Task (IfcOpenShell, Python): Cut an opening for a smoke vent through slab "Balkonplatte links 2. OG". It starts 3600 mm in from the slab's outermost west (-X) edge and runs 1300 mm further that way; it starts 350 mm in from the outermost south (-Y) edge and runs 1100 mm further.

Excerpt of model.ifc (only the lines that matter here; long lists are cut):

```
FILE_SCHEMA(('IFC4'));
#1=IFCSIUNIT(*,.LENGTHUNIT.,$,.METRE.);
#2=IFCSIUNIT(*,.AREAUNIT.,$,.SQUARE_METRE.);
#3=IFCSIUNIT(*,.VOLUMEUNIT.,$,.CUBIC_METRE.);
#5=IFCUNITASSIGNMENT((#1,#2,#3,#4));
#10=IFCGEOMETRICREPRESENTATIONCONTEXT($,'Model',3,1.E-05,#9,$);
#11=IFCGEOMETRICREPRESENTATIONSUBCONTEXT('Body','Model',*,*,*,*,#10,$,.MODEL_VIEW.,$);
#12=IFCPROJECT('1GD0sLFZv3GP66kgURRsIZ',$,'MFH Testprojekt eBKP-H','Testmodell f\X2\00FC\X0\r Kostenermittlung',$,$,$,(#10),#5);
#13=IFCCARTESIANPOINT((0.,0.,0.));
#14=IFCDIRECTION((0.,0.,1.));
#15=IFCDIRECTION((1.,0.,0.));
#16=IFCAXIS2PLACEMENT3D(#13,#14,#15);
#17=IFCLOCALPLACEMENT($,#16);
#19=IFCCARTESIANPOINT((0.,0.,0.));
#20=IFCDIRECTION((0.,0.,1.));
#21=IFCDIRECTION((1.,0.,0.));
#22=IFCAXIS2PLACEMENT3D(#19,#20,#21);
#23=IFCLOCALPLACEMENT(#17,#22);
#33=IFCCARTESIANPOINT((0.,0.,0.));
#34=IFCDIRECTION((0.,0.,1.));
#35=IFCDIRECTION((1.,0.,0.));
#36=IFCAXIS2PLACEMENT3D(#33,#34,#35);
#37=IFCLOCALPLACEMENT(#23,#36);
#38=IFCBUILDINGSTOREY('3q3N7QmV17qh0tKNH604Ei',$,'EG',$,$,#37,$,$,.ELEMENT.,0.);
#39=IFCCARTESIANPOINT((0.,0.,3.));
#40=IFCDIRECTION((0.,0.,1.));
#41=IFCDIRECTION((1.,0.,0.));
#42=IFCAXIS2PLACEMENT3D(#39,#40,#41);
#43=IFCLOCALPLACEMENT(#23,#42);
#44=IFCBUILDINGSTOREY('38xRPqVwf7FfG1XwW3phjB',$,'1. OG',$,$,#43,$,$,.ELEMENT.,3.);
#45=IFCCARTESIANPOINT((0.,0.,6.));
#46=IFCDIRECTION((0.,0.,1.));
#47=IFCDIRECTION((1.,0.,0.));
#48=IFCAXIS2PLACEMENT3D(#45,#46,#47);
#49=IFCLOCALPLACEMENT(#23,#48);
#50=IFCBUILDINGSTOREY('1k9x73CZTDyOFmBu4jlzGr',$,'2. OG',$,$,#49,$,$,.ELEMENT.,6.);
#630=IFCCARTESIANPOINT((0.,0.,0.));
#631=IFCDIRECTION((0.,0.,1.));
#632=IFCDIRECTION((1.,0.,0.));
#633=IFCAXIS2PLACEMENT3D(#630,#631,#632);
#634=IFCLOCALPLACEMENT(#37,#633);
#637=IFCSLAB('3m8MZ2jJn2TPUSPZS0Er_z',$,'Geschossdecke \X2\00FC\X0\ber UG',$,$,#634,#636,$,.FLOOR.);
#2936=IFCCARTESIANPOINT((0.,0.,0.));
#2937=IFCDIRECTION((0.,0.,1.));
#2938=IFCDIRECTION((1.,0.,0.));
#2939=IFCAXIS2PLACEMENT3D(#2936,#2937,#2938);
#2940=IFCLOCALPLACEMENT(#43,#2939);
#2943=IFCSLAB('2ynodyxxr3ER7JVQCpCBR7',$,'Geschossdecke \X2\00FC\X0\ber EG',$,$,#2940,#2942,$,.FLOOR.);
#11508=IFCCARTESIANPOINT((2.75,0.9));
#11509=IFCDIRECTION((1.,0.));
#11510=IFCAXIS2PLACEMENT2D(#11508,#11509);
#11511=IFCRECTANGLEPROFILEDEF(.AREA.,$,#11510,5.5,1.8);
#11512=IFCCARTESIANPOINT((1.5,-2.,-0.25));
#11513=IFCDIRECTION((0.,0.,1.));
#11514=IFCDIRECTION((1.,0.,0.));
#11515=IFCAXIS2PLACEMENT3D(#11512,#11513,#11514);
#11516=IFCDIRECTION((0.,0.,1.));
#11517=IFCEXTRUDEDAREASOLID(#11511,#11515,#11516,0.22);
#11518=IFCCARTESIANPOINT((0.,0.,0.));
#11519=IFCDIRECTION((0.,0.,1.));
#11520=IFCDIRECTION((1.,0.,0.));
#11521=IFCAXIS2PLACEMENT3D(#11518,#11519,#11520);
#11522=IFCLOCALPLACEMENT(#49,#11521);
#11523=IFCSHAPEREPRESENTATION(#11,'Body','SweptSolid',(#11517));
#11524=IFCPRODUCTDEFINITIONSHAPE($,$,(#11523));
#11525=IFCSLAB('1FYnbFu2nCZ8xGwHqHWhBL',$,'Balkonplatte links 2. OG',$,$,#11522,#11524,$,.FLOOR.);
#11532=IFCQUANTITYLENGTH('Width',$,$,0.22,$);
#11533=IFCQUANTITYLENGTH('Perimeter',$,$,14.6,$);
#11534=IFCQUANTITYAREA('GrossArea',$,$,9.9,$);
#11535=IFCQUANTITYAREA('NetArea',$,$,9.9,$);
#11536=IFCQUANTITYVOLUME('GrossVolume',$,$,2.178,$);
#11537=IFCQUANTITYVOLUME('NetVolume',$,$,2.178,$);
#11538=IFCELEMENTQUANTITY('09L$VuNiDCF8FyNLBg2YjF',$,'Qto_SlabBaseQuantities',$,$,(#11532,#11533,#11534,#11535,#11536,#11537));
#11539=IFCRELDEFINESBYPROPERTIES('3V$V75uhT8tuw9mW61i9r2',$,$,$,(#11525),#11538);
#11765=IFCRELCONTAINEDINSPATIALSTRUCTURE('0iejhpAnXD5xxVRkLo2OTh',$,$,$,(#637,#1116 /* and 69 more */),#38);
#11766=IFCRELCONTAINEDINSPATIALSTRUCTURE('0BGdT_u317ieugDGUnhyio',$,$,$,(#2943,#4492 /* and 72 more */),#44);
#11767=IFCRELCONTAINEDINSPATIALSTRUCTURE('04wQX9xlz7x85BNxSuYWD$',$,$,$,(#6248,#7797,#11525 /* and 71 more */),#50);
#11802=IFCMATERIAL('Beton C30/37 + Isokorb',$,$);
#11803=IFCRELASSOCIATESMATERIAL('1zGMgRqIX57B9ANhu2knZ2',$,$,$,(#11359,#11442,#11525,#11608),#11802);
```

```python
import numpy as np
import ifcopenshell
import ifcopenshell.api.feature
import ifcopenshell.api.geometry
import ifcopenshell.api.pset
import ifcopenshell.api.root
import ifcopenshell.geom
import ifcopenshell.util.element
import ifcopenshell.util.placement
import ifcopenshell.util.representation
import ifcopenshell.util.shape
import ifcopenshell.util.unit

model = ifcopenshell.open("model.ifc")
unit_scale = ifcopenshell.util.unit.calculate_unit_scale(model)
area_scale = ifcopenshell.util.unit.calculate_unit_scale(model, "AREAUNIT")
volume_scale = ifcopenshell.util.unit.calculate_unit_scale(model, "VOLUMEUNIT")
settings = ifcopenshell.geom.settings()


def volume(element):
    """Net volume in cubic metres, openings subtracted."""
    shape = ifcopenshell.geom.create_shape(settings, element)
    return ifcopenshell.util.shape.get_volume(shape.geometry)


slab = model.by_guid("1FYnbFu2nCZ8xGwHqHWhBL")
before = volume(slab)

# Extent in the slab's own axes, in metres. The edges named are its -X and -Y sides.
slab_shape = ifcopenshell.geom.create_shape(settings, slab)
vertices = ifcopenshell.util.shape.get_vertices(slab_shape.geometry)
x_min, y_min, bottom = vertices.min(axis=0)
top = vertices[:, 2].max()

opening = ifcopenshell.api.root.create_entity(model, ifc_class="IfcOpeningElement", name="Smoke vent opening", predefined_type="OPENING")
context = ifcopenshell.util.representation.get_context(model, "Model", "Body", "MODEL_VIEW")
width, depth = 1.3, 1.1
outline = [(0.0, 0.0), (width, 0.0), (width, depth), (0.0, depth), (0.0, 0.0)]
# Overshoot both faces by 50 mm so the cut is clean.
shape = ifcopenshell.api.geometry.add_slab_representation(
    model, context=context, depth=top - bottom + 0.1, polyline=outline
)
ifcopenshell.api.geometry.assign_representation(model, product=opening, representation=shape)

matrix = ifcopenshell.util.placement.get_local_placement(slab.ObjectPlacement)
matrix[:, 3] = matrix @ np.append(np.array([x_min + 3.6, y_min + 0.35, bottom - 0.05]) / unit_scale, 1.0)
ifcopenshell.api.geometry.edit_object_placement(model, product=opening, matrix=matrix, is_si=False)
ifcopenshell.api.feature.add_feature(model, feature=opening, element=slab)

after = volume(slab)

# Update the slab's stored quantities.
qto = model.by_id(ifcopenshell.util.element.get_pset(slab, "Qto_SlabBaseQuantities", should_inherit=False)["id"])
ifcopenshell.api.pset.edit_qto(model, qto=qto, properties={
    "NetArea": after / (top - bottom) / area_scale,
    "NetVolume": after / volume_scale,
})

print(f"slab volume {before:.3f} -> {after:.3f} m3")

model.write("model_edited.ifc")
```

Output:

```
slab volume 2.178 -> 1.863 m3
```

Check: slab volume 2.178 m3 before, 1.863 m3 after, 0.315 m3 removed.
